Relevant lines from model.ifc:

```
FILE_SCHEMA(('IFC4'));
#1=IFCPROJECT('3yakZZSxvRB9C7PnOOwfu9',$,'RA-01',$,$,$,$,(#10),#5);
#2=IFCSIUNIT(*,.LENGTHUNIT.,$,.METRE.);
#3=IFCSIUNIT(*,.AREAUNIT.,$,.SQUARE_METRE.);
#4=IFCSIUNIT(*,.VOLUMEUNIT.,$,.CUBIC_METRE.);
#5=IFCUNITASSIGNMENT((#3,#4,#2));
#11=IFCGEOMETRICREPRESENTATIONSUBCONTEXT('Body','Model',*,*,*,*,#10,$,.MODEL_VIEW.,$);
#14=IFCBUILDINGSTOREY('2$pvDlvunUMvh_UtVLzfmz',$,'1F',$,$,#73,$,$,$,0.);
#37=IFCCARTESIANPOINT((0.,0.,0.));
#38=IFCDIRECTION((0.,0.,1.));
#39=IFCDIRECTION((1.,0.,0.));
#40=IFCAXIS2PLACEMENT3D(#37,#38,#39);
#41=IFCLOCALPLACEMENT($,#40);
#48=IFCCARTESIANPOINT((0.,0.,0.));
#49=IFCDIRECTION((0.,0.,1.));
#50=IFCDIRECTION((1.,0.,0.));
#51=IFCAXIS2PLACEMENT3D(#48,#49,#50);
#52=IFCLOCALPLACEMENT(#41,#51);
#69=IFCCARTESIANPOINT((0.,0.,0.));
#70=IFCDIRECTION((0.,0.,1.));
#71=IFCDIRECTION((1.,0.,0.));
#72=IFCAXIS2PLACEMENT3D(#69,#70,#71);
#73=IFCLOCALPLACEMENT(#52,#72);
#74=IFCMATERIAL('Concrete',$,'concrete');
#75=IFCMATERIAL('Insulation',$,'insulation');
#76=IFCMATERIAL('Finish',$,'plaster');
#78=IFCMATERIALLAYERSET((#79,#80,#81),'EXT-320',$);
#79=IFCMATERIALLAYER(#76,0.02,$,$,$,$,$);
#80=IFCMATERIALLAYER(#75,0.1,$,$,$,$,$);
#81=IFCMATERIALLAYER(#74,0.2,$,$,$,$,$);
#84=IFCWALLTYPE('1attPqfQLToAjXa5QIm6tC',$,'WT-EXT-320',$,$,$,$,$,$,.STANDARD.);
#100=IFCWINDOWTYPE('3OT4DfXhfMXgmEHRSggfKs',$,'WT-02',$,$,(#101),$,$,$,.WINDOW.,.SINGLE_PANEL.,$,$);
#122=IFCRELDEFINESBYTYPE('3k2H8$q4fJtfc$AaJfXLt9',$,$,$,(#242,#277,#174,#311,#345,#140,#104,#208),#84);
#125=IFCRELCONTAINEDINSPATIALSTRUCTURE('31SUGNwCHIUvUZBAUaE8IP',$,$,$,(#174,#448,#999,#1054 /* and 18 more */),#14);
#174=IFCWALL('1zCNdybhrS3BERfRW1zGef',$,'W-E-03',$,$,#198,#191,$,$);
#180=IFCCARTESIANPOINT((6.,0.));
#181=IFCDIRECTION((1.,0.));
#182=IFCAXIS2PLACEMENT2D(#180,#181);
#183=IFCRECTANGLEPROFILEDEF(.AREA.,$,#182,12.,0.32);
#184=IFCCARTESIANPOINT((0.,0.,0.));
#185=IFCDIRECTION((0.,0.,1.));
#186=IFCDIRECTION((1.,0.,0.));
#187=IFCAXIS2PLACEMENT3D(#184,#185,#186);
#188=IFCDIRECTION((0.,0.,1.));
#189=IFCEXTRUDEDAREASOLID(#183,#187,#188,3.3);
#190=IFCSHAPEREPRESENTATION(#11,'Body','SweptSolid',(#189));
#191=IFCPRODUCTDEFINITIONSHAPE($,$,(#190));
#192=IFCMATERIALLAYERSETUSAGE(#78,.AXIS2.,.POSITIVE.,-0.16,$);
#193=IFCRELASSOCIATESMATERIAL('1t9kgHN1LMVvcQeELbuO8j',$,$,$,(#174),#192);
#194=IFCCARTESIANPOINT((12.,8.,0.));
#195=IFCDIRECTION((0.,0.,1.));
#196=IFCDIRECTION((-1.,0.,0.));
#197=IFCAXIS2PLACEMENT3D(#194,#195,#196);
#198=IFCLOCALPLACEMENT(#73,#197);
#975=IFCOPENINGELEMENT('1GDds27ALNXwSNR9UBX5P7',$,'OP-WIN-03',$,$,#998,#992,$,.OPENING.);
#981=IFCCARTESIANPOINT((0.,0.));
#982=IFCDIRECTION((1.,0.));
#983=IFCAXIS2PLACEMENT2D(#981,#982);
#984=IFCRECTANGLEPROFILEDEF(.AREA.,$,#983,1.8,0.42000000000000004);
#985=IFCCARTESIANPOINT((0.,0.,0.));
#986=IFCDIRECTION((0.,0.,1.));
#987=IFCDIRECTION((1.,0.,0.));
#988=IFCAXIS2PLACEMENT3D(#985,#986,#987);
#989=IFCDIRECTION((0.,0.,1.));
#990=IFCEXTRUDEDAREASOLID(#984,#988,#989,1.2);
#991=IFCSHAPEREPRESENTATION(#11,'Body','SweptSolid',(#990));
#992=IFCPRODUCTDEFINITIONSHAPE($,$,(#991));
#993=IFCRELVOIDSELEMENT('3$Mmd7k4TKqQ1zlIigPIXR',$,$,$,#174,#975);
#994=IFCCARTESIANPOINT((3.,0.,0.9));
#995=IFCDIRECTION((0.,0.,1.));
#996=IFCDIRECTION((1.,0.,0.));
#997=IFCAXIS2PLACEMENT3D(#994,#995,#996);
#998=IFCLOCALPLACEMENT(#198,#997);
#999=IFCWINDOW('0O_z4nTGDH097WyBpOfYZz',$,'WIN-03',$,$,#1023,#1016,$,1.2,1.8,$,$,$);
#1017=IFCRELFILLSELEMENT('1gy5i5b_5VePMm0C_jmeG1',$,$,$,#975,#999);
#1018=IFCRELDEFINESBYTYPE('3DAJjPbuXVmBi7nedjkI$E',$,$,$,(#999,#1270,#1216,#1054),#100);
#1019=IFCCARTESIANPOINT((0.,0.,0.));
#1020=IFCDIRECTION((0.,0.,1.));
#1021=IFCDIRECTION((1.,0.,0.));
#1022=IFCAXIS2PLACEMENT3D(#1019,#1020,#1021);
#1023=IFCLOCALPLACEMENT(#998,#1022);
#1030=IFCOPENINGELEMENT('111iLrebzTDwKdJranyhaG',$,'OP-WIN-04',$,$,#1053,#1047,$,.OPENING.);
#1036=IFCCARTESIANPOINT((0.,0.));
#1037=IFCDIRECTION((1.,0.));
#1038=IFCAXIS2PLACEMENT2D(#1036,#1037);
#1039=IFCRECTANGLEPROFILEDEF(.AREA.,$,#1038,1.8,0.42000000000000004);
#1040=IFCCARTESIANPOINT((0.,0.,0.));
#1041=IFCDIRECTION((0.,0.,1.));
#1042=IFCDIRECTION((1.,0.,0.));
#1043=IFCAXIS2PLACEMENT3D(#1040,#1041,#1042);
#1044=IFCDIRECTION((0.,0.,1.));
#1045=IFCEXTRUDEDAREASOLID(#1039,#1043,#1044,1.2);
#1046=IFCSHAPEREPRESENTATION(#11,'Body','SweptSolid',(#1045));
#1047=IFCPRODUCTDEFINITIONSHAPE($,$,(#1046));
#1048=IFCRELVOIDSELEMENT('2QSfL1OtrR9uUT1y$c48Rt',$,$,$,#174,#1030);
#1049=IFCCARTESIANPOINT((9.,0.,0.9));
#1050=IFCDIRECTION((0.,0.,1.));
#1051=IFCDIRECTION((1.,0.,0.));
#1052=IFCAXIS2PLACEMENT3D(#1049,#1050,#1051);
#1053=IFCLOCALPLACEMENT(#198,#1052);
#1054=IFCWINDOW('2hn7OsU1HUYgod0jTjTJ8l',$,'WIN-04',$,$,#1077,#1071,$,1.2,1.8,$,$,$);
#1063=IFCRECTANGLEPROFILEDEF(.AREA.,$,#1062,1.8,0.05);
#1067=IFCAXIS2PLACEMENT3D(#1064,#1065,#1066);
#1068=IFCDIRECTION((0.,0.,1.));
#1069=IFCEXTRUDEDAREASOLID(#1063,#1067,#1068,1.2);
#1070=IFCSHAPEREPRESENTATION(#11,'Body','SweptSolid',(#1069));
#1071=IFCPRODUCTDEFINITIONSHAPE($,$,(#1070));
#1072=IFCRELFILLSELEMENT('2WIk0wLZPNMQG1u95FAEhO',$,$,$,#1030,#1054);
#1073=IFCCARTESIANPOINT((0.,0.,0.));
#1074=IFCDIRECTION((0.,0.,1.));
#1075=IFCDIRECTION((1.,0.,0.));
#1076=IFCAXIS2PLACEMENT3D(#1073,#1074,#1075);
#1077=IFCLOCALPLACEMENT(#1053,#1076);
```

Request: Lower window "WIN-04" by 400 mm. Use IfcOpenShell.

```python
import numpy as np
import ifcopenshell
import ifcopenshell.api.geometry
import ifcopenshell.util.placement
import ifcopenshell.util.unit

model = ifcopenshell.open("model.ifc")
unit_scale = ifcopenshell.util.unit.calculate_unit_scale(model)

window = model.by_guid("2hn7OsU1HUYgod0jTjTJ8l")
opening = window.FillsVoids[0].RelatingOpeningElement
dz = -0.4

shift = np.array([0.0, 0.0, dz])
# The window is placed relative to its opening, so it follows when the opening moves.
matrix = ifcopenshell.util.placement.get_local_placement(opening.ObjectPlacement)
matrix[:3, 3] += shift
ifcopenshell.api.geometry.edit_object_placement(
    model, product=opening, matrix=matrix, is_si=False, should_transform_children=True
)

print(f"moved by {dz * unit_scale:+.3f} m")

model.write("model_rev.ifc")
```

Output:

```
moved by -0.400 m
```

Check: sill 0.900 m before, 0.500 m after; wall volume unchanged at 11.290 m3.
